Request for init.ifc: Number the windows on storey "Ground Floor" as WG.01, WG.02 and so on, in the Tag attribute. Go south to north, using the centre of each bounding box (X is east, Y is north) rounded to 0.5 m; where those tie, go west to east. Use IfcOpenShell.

First a look at what the model holds.

```python
import ifcopenshell
import ifcopenshell.util.element
import ifcopenshell.util.placement

model = ifcopenshell.open("init.ifc")
print(model.schema)
storey = next(s for s in model.by_type("IfcBuildingStorey") if s.Name == "Ground Floor")
windows = [e for e in ifcopenshell.util.element.get_decomposition(storey) if e.is_a("IfcWindow")]
for e in sorted(windows, key=lambda e: e.id()):
    origin = ifcopenshell.util.placement.get_local_placement(e.ObjectPlacement)[:3, 3]
    print(e.id(), e.Tag, e.Name, origin.round(2) + 0.0, sep=" | ")
```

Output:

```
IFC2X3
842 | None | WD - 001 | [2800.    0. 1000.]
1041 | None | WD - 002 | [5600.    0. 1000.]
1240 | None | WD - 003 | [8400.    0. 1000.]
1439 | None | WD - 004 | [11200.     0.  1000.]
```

```python
import ifcopenshell
import ifcopenshell.geom
import ifcopenshell.util.element
import ifcopenshell.util.shape

model = ifcopenshell.open("init.ifc")
settings = ifcopenshell.geom.settings()
settings.set("use-world-coords", True)


def centre(element):
    shape = ifcopenshell.geom.create_shape(settings, element)
    return ifcopenshell.util.shape.get_bbox_centroid(shape.geometry)


storey = next(s for s in model.by_type("IfcBuildingStorey") if s.Name == "Ground Floor")
windows = [e for e in ifcopenshell.util.element.get_decomposition(storey) if e.is_a("IfcWindow")]

# Insertion points can sit at a corner or the storey origin, so sort by the geometry (in metres).
centres = {e: centre(e) for e in windows}
windows.sort(key=lambda e: (round(centres[e][1] / 0.5), centres[e][0]))

for i, e in enumerate(windows, start=1):
    number = f"WG.{i:02d}"
    e.Tag = number
    print(e.id(), number)

model.write("init_updated.ifc")
```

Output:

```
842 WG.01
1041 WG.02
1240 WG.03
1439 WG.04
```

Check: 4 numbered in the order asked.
